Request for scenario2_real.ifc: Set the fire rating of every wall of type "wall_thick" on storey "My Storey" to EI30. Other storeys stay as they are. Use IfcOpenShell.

First a look at what the model holds.

```python
import ifcopenshell
import ifcopenshell.util.element

model = ifcopenshell.open("scenario2_real.ifc")
print(model.schema)
storey = next(s for s in model.by_type("IfcBuildingStorey") if s.Name == "My Storey")
walls = [e for e in ifcopenshell.util.element.get_decomposition(storey) if e.is_a("IfcWall")]
seen = {}
for e in walls:
    element_type = ifcopenshell.util.element.get_type(e)
    key = (element_type.Name if element_type != e and element_type else None, ifcopenshell.util.element.get_pset(e, "Pset_WallCommon", "FireRating"))
    seen[key] = seen.get(key, 0) + 1
for (name, value), count in sorted(seen.items(), key=str):
    print(count, "x", name, "|", value)
```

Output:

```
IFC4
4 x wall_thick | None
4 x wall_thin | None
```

```python
import ifcopenshell
import ifcopenshell.api.pset
import ifcopenshell.util.element

model = ifcopenshell.open("scenario2_real.ifc")

storey = next(s for s in model.by_type("IfcBuildingStorey") if s.Name == "My Storey")
walls = [e for e in ifcopenshell.util.element.get_decomposition(storey) if e.is_a("IfcWall")]

count = 0
for e in walls:
    element_type = ifcopenshell.util.element.get_type(e)
    if element_type in (None, e) or element_type.Name != "wall_thick":
        continue
    # add_pset returns the element's existing set when there is one.
    pset = ifcopenshell.api.pset.add_pset(model, product=e, name="Pset_WallCommon")
    ifcopenshell.api.pset.edit_pset(model, pset=pset, properties={"FireRating": "EI30"})
    count += 1

print(count, "walls updated")

model.write("scenario2_real-out.ifc")
```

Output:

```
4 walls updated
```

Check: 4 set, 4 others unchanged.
